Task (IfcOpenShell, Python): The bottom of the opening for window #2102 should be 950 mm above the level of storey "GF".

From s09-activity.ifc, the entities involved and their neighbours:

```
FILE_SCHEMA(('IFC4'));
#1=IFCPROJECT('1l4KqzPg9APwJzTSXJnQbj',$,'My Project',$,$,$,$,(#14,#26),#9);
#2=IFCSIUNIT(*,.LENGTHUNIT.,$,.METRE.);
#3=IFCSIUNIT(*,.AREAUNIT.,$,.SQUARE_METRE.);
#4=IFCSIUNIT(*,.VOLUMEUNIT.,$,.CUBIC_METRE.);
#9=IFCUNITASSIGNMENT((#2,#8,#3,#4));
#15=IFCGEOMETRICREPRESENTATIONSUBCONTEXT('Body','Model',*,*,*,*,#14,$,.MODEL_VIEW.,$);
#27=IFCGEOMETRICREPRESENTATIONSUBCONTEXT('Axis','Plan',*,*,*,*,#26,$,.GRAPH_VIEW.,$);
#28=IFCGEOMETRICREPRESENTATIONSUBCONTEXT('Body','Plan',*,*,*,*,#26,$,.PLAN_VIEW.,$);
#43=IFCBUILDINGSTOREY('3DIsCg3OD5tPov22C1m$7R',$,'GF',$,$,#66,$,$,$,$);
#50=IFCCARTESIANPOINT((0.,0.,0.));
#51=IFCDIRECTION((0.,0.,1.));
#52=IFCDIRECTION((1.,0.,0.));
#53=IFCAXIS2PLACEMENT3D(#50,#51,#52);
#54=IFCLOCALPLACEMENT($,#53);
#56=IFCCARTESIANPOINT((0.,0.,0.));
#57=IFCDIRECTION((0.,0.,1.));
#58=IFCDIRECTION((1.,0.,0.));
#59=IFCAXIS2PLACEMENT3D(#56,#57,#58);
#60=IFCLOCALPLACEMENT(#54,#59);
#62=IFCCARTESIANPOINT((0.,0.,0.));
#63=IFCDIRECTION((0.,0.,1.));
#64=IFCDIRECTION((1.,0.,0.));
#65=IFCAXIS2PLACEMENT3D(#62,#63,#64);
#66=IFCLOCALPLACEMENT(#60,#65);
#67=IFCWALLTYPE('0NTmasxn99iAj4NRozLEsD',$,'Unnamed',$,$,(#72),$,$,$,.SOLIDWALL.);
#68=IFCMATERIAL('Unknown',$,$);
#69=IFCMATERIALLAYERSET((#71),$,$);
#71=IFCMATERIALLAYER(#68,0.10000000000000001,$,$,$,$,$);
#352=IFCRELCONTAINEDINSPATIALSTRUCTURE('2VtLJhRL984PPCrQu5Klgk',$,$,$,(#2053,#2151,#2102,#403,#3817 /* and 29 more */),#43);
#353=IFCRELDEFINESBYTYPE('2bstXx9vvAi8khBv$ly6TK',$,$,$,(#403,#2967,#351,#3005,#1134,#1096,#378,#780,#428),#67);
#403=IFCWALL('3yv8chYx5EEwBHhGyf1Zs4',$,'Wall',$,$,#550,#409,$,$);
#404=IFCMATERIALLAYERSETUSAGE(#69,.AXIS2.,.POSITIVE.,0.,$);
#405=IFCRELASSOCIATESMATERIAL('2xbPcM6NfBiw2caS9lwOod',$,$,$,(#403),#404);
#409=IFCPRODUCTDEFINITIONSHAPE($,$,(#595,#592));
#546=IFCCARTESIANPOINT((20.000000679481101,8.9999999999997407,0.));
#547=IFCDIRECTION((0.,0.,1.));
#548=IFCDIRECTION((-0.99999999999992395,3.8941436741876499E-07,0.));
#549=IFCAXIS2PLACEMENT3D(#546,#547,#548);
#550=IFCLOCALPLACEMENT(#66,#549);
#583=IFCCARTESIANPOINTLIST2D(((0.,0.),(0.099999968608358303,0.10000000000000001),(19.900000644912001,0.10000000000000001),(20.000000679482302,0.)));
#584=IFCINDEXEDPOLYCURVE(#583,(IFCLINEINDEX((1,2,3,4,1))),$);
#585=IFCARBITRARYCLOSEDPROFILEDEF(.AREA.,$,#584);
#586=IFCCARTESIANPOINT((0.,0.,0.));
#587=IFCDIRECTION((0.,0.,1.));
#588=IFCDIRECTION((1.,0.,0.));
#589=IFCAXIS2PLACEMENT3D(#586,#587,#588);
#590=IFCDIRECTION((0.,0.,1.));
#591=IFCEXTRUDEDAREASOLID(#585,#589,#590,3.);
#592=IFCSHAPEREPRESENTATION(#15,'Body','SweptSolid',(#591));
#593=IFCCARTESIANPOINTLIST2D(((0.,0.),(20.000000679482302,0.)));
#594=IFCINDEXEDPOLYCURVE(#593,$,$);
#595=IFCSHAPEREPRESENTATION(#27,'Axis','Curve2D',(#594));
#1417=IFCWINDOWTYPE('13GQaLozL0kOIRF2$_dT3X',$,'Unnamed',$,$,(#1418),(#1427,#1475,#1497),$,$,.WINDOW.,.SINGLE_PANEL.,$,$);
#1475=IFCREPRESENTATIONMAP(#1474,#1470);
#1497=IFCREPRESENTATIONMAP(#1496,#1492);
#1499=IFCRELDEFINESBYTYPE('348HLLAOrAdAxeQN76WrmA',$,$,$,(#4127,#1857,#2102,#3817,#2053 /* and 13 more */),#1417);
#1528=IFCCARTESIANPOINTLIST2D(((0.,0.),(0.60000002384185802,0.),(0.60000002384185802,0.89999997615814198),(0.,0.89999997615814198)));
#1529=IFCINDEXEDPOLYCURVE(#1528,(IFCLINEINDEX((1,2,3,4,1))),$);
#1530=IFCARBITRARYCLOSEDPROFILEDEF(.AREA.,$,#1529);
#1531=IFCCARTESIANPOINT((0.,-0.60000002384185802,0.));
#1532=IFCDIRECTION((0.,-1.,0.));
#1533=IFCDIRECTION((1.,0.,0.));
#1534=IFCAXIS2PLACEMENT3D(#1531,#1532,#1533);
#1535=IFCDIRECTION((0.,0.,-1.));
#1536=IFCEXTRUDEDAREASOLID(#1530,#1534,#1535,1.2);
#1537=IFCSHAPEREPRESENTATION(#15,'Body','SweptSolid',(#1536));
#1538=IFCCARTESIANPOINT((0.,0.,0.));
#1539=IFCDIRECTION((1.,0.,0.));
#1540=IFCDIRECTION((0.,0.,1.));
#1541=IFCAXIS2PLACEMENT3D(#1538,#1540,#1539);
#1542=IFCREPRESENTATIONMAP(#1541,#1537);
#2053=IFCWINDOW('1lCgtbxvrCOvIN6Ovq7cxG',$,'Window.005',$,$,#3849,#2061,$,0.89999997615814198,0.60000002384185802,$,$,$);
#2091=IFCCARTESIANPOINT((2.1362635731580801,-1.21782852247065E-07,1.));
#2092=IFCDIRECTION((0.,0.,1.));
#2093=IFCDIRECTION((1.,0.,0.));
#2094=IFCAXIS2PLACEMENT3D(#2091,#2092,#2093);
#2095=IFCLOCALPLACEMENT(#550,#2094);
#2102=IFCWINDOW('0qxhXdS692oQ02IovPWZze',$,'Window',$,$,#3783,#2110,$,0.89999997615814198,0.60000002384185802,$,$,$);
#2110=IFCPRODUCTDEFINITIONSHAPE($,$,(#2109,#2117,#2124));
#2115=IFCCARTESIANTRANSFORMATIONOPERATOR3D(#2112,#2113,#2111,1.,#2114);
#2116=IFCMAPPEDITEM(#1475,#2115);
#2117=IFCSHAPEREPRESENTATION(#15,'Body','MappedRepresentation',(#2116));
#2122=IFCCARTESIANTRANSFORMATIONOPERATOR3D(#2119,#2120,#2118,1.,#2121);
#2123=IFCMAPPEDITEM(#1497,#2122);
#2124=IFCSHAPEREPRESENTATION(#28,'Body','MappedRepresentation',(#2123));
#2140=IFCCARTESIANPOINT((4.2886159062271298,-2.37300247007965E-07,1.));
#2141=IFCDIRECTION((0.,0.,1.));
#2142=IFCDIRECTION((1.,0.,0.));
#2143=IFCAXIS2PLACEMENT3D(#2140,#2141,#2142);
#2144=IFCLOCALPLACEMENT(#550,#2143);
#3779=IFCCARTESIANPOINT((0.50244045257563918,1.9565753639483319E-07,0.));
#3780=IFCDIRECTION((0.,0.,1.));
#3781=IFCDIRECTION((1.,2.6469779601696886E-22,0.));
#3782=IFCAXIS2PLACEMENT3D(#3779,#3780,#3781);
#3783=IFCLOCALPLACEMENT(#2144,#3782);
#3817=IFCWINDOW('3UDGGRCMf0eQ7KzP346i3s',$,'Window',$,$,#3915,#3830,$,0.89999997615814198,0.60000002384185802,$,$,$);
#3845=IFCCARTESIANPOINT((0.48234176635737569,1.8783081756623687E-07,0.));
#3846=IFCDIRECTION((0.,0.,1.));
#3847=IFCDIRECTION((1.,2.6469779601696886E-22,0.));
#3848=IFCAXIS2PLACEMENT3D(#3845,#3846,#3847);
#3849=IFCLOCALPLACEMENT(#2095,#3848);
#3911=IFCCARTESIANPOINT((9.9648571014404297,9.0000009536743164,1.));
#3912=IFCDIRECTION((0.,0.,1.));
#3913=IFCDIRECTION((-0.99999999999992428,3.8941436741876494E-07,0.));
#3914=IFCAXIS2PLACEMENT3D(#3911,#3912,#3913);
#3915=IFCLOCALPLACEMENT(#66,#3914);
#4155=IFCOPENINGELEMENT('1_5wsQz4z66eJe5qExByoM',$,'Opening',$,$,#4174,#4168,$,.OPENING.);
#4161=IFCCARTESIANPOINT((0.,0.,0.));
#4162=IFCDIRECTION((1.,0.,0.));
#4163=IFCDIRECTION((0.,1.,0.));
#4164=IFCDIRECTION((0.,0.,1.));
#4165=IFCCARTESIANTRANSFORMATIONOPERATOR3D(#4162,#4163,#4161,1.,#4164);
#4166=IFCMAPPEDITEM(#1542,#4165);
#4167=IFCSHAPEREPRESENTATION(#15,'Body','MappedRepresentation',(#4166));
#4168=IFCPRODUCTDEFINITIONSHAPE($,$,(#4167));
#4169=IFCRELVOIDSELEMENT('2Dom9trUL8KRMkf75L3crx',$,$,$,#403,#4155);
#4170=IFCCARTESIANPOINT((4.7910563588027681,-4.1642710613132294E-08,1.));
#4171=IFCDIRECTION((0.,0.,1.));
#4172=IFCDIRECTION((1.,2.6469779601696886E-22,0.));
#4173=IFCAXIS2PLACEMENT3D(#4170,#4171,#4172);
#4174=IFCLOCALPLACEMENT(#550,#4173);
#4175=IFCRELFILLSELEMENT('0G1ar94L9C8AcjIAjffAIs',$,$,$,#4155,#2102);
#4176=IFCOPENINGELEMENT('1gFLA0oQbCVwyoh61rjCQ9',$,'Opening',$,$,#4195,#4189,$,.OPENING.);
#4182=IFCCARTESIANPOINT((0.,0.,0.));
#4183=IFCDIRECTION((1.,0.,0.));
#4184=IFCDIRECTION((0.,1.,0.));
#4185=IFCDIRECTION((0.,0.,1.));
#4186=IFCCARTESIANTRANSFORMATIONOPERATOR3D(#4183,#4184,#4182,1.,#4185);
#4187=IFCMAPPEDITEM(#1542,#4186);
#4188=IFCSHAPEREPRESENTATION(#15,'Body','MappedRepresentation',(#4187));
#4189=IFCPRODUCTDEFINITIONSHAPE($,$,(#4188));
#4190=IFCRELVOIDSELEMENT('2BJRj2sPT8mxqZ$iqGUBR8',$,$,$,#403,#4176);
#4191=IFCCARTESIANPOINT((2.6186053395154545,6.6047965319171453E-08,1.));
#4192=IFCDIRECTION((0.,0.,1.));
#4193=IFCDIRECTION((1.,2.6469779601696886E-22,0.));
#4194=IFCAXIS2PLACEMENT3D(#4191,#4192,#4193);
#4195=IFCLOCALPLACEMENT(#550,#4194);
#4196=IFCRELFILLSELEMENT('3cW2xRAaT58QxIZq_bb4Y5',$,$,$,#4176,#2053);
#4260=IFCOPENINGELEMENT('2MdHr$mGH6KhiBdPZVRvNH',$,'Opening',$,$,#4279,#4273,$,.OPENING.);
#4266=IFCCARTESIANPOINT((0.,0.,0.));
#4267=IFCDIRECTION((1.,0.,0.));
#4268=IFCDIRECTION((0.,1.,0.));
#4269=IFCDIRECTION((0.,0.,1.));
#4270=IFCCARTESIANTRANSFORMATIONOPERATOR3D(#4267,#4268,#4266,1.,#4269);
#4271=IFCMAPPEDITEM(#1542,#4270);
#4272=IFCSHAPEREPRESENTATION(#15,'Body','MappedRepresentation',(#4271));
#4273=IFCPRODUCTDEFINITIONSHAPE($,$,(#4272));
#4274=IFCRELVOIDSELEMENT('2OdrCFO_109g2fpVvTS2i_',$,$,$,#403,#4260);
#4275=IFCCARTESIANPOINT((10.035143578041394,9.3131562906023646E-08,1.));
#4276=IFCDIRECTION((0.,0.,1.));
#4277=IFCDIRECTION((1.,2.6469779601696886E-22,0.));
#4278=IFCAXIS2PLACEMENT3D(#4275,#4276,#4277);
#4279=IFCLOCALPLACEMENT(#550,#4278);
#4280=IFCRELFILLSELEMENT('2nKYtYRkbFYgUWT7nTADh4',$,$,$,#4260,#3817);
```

```python
import numpy as np
import ifcopenshell
import ifcopenshell.api.geometry
import ifcopenshell.geom
import ifcopenshell.util.element
import ifcopenshell.util.placement
import ifcopenshell.util.shape
import ifcopenshell.util.unit

model = ifcopenshell.open("s09-activity.ifc")
unit_scale = ifcopenshell.util.unit.calculate_unit_scale(model)

window = model.by_guid("0qxhXdS692oQ02IovPWZze")
opening = window.FillsVoids[0].RelatingOpeningElement
storey = ifcopenshell.util.element.get_container(window, ifc_class="IfcBuildingStorey")
level = ifcopenshell.util.placement.get_local_placement(storey.ObjectPlacement)[2, 3]

# The opening's origin need not be at the sill, so measure its lowest point.
shape = ifcopenshell.geom.create_shape(ifcopenshell.geom.settings(), opening)
bottom = ifcopenshell.util.shape.get_shape_bottom_elevation(shape, shape.geometry) / unit_scale
dz = level + 0.95 - bottom

shift = np.array([0.0, 0.0, dz])
# The window is not placed relative to its opening, so move both.
for product in (opening, window):
    matrix = ifcopenshell.util.placement.get_local_placement(product.ObjectPlacement)
    matrix[:3, 3] += shift
    ifcopenshell.api.geometry.edit_object_placement(model, product=product, matrix=matrix, is_si=False)

print(f"moved by {dz * unit_scale:+.3f} m")

model.write("s09-activity_updated.ifc")
```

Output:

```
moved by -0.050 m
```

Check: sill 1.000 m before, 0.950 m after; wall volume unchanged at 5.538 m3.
